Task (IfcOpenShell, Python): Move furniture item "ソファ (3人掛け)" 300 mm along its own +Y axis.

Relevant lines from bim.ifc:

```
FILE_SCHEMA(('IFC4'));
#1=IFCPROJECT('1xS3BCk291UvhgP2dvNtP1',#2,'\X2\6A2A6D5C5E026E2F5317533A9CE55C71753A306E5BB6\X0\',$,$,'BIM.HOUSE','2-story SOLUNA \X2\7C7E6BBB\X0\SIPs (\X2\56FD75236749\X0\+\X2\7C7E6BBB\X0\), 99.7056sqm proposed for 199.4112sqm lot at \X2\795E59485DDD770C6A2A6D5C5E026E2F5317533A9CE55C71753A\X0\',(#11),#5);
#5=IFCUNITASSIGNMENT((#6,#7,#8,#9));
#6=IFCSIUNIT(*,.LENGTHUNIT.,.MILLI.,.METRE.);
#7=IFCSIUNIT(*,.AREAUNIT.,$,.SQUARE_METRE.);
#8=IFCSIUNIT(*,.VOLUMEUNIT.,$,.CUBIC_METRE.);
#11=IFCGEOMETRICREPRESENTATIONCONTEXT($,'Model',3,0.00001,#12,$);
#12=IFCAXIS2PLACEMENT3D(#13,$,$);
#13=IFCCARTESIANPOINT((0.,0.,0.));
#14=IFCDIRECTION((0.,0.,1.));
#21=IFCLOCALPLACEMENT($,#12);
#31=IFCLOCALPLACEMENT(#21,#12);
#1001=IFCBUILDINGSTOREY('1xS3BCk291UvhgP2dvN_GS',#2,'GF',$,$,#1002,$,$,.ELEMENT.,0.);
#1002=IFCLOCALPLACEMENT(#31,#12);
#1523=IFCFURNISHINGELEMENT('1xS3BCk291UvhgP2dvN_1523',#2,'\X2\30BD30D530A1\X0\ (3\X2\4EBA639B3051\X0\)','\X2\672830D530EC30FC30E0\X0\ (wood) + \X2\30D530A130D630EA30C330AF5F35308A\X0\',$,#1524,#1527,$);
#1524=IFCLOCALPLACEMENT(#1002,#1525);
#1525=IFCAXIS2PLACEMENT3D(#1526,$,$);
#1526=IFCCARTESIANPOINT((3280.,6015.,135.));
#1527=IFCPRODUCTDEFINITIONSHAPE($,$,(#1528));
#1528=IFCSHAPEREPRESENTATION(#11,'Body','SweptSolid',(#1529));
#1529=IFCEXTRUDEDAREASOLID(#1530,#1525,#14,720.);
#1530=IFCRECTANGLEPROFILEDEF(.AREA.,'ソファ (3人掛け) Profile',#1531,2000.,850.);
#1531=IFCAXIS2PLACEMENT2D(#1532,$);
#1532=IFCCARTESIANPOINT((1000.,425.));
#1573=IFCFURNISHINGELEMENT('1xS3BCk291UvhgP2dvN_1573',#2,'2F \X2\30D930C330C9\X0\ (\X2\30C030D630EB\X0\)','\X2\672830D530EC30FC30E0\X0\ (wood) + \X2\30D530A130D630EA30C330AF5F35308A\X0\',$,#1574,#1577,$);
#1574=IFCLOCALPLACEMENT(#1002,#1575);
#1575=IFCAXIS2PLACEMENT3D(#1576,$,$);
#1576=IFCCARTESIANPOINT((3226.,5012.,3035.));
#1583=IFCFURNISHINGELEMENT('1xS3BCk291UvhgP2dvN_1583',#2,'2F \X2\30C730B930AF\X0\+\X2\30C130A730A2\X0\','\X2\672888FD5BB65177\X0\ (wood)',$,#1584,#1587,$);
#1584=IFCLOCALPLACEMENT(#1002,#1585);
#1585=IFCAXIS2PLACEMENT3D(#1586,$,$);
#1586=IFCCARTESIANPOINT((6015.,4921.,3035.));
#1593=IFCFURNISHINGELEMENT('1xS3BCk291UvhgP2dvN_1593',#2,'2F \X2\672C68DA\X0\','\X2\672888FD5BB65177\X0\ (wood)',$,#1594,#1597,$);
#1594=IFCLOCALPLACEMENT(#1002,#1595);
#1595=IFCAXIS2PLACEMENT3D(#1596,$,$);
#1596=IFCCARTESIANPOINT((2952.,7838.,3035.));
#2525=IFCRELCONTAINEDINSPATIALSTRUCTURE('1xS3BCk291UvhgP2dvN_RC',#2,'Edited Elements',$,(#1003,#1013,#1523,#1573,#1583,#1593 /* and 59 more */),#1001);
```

```python
import ifcopenshell
import ifcopenshell.api.geometry
import ifcopenshell.util.placement
import ifcopenshell.util.unit

model = ifcopenshell.open("bim.ifc")
unit_scale = ifcopenshell.util.unit.calculate_unit_scale(model)

item = model.by_id(1523)
matrix = ifcopenshell.util.placement.get_local_placement(item.ObjectPlacement)
matrix[:3, 3] += matrix[:3, 1] * 0.3 / unit_scale
ifcopenshell.api.geometry.edit_object_placement(model, product=item, matrix=matrix, is_si=False)

print(ifcopenshell.util.placement.get_local_placement(item.ObjectPlacement).round(3) + 0.0)

model.write("bim_rev.ifc")
```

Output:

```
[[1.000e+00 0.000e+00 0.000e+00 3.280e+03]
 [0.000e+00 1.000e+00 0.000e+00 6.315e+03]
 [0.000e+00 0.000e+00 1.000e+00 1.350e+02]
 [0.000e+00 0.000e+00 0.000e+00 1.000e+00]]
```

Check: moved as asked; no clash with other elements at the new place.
